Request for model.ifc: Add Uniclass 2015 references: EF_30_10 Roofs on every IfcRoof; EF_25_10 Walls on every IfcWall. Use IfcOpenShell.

First a look at what the model holds.

```python
import ifcopenshell

model = ifcopenshell.open("model.ifc")
print(model.schema)
print("classifications:", [c.Name for c in model.by_type("IfcClassification")])
for ifc_class in ("IfcDoor", "IfcRoof", "IfcStair", "IfcWall", "IfcWindow"):
    print(ifc_class, len(model.by_type(ifc_class)))
```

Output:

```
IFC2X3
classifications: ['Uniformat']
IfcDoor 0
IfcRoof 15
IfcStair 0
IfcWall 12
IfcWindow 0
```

```python
import ifcopenshell
import ifcopenshell.api.classification

model = ifcopenshell.open("model.ifc")

# IFC2X3 requires Source and Edition and has no link from the project to the system.
system = model.create_entity("IfcClassification", Source="NBS", Edition="2015", Name="Uniclass 2015")

codes = {
    "IfcRoof": ("EF_30_10", "Roofs"),
    "IfcWall": ("EF_25_10", "Walls"),
}
for ifc_class, (code, name) in codes.items():
    products = model.by_type(ifc_class)
    ifcopenshell.api.classification.add_reference(
        model, products=products, classification=system, identification=code, name=name
    )
    print(code, len(products))

model.write("model_v2.ifc")
```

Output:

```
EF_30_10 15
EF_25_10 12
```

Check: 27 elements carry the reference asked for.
